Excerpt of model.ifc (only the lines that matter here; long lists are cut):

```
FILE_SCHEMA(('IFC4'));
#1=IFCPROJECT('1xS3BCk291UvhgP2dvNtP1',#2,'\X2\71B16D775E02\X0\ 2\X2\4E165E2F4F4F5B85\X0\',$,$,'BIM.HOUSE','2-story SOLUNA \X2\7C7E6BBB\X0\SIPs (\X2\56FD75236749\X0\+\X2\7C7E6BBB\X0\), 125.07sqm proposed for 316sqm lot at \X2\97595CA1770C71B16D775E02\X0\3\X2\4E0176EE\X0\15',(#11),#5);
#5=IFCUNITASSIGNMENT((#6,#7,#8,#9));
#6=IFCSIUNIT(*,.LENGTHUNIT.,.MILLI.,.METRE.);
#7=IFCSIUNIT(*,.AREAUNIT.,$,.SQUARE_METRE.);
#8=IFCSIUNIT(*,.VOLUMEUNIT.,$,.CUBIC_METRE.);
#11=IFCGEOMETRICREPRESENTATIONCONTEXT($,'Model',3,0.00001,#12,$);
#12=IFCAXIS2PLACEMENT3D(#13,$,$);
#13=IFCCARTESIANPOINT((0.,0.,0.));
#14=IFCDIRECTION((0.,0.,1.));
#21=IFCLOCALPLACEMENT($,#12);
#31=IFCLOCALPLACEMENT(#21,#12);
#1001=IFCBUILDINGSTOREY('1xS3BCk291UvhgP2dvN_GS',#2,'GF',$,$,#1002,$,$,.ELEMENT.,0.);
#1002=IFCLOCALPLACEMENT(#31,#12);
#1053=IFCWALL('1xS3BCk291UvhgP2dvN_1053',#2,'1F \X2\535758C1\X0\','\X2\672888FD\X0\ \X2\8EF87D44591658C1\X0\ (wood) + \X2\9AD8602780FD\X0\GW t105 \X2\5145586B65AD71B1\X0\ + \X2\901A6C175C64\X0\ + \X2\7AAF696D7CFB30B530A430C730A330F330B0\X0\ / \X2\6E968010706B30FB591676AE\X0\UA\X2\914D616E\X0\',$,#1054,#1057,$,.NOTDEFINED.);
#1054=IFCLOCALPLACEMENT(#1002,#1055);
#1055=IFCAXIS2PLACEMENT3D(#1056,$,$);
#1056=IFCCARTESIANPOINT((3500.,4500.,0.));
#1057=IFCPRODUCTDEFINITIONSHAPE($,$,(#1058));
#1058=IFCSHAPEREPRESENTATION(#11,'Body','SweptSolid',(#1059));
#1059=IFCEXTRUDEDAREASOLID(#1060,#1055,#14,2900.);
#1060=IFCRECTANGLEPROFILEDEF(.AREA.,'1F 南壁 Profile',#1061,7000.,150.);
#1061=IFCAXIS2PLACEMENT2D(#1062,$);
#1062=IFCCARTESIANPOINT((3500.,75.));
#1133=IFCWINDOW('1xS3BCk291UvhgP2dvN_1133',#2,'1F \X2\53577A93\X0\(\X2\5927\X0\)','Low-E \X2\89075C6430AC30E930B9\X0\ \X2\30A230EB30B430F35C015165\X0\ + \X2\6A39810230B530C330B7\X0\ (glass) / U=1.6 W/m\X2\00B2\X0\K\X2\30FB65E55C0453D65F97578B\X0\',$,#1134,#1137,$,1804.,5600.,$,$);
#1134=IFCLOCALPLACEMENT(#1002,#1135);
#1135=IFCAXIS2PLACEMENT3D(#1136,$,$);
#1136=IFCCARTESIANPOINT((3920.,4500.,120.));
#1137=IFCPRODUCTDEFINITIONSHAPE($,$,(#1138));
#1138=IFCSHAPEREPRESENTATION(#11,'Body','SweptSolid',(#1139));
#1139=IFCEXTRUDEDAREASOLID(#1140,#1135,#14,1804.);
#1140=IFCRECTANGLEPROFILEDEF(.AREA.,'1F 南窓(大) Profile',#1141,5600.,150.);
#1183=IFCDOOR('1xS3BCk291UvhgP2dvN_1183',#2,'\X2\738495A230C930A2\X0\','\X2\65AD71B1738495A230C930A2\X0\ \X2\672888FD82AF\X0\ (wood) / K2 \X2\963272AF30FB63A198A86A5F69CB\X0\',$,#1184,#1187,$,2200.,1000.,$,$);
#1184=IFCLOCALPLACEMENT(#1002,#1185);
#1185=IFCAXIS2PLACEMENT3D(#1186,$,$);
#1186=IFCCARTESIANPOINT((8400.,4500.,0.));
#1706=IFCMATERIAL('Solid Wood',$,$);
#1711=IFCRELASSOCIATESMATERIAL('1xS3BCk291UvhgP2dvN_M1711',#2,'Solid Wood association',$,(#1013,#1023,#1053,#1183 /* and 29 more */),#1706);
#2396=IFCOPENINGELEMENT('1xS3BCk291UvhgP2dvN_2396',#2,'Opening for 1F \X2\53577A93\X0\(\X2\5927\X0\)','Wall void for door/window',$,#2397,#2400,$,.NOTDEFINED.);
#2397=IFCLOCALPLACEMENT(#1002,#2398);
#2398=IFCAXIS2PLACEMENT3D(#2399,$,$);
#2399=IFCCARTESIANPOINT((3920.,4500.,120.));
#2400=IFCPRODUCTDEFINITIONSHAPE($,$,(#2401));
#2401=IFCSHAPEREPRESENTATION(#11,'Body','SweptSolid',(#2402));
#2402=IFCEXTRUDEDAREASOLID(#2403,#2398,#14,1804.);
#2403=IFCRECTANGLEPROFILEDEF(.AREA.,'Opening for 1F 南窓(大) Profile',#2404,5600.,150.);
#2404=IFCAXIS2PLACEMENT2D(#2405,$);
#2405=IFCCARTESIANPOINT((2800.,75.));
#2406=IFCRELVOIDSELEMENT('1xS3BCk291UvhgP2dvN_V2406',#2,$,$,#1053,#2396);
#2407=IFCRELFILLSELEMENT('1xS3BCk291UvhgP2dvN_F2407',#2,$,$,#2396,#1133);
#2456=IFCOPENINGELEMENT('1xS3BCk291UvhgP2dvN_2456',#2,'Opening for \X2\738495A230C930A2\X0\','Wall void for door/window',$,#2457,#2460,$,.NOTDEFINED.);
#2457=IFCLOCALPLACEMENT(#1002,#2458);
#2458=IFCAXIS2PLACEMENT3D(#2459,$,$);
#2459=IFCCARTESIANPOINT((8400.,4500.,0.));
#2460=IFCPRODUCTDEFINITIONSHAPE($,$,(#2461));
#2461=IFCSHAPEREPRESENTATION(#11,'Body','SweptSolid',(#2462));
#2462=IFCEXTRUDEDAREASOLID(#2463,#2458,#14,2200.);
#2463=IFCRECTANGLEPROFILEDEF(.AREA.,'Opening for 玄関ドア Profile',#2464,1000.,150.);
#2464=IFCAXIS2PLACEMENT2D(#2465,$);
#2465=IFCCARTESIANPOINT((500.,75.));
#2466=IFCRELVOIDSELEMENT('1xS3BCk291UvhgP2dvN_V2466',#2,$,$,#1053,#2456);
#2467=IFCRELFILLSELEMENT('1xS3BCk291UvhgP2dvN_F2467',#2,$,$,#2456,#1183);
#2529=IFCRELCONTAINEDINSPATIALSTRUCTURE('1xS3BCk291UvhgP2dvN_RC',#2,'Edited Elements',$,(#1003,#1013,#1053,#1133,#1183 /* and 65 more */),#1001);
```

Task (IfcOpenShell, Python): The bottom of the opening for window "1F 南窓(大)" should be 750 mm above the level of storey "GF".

```python
import numpy as np
import ifcopenshell
import ifcopenshell.api.geometry
import ifcopenshell.geom
import ifcopenshell.util.element
import ifcopenshell.util.placement
import ifcopenshell.util.shape
import ifcopenshell.util.unit

model = ifcopenshell.open("model.ifc")
unit_scale = ifcopenshell.util.unit.calculate_unit_scale(model)

window = model.by_guid("1xS3BCk291UvhgP2dvN_1133")
opening = window.FillsVoids[0].RelatingOpeningElement
storey = ifcopenshell.util.element.get_container(window, ifc_class="IfcBuildingStorey")
level = ifcopenshell.util.placement.get_local_placement(storey.ObjectPlacement)[2, 3]

# The opening's origin need not be at the sill, so measure its lowest point.
shape = ifcopenshell.geom.create_shape(ifcopenshell.geom.settings(), opening)
bottom = ifcopenshell.util.shape.get_shape_bottom_elevation(shape, shape.geometry) / unit_scale
dz = level + 750.0 - bottom

shift = np.array([0.0, 0.0, dz])
# The window is not placed relative to its opening, so move both.
for product in (opening, window):
    matrix = ifcopenshell.util.placement.get_local_placement(product.ObjectPlacement)
    matrix[:3, 3] += shift
    ifcopenshell.api.geometry.edit_object_placement(model, product=product, matrix=matrix, is_si=False)

print(f"moved by {dz * unit_scale:+.3f} m")

model.write("model_rev.ifc")
```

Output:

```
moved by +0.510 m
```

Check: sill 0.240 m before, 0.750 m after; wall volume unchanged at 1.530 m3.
